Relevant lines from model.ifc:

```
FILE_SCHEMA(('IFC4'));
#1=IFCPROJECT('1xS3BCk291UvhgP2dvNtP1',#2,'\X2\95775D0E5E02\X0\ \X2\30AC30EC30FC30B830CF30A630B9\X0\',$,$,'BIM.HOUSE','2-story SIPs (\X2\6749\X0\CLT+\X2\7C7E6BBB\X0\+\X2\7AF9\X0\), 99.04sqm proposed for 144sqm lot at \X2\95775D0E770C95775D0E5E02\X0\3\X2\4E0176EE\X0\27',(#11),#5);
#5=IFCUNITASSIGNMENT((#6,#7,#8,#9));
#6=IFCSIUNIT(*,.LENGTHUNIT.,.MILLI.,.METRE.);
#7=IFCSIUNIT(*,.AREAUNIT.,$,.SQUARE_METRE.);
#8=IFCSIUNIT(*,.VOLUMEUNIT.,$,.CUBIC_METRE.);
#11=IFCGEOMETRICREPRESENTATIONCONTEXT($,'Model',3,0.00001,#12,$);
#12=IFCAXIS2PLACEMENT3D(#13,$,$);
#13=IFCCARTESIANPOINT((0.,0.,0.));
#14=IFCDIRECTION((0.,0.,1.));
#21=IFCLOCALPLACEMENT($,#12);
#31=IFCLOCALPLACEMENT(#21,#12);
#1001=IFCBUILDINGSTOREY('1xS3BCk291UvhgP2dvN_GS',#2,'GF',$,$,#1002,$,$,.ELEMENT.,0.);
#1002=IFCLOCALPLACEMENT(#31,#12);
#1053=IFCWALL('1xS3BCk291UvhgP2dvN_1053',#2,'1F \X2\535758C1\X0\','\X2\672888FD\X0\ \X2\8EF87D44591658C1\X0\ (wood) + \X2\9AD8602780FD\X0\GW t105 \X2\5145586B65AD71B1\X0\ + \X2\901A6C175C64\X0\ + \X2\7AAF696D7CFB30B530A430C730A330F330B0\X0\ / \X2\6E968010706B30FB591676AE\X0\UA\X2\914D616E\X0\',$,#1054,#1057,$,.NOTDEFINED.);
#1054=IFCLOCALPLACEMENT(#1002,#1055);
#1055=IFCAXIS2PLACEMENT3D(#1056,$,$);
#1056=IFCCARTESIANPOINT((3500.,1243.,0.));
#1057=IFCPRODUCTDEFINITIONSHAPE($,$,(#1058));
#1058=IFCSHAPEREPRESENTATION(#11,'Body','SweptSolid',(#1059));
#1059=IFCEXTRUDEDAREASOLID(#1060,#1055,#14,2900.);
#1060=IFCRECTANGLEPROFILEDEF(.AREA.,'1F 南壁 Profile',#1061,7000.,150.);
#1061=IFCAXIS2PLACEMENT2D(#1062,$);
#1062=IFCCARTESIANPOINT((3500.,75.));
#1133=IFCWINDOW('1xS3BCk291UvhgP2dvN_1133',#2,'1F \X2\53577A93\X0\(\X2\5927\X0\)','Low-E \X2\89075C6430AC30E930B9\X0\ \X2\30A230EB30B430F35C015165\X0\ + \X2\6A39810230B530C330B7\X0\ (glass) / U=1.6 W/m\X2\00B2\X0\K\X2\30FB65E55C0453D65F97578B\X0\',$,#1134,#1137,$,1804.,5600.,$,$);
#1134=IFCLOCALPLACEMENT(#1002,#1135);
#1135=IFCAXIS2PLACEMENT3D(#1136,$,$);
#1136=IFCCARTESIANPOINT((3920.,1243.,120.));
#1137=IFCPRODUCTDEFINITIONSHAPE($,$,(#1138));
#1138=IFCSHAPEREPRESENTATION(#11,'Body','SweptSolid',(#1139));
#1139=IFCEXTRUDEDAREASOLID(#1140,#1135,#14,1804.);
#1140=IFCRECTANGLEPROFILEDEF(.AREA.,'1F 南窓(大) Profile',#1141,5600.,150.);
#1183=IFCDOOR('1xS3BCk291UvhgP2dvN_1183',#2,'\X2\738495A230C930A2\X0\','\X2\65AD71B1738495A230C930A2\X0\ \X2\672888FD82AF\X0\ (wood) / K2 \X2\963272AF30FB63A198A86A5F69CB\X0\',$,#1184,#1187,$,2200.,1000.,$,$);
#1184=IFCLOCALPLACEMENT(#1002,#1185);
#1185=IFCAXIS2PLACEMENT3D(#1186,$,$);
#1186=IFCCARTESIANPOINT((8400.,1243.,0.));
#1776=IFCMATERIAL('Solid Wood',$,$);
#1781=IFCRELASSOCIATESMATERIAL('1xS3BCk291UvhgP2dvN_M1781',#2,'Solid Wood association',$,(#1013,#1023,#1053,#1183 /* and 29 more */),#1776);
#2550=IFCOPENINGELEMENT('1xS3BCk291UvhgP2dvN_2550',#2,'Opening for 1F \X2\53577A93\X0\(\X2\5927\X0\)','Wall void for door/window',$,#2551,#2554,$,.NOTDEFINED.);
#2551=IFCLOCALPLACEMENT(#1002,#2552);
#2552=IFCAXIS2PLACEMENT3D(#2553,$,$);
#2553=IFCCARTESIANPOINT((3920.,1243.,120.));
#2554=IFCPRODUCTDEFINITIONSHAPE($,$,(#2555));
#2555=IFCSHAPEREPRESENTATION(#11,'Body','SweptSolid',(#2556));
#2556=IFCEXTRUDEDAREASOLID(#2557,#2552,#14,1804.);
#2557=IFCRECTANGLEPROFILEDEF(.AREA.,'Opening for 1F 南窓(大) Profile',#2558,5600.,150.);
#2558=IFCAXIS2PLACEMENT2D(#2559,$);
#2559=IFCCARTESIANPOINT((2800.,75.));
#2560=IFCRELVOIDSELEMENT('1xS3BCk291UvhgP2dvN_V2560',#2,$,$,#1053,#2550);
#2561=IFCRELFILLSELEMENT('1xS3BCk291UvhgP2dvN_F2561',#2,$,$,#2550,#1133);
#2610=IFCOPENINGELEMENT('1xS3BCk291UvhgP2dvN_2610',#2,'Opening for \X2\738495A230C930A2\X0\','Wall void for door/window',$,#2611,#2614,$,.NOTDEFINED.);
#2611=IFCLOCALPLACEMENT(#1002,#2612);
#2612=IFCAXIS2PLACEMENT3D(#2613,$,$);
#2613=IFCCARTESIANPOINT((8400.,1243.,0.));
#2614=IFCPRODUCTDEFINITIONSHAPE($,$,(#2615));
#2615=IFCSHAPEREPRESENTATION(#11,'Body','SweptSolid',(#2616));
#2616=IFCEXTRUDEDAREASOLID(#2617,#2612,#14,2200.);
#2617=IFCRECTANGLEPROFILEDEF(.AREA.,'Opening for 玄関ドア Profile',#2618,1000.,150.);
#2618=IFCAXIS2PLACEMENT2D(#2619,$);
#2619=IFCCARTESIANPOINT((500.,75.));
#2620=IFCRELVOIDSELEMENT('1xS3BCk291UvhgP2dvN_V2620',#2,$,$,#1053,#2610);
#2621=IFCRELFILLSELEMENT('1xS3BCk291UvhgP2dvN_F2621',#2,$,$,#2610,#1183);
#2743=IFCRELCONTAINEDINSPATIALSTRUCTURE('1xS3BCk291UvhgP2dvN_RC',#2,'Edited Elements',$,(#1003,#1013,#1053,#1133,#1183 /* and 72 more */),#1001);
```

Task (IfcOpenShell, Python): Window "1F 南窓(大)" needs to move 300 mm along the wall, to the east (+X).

```python
import ifcopenshell
import ifcopenshell.api.geometry
import ifcopenshell.util.placement

model = ifcopenshell.open("model.ifc")

window = model.by_guid("1xS3BCk291UvhgP2dvN_1133")
opening = window.FillsVoids[0].RelatingOpeningElement
wall = opening.VoidsElements[0].RelatingBuildingElement

wall_matrix = ifcopenshell.util.placement.get_local_placement(wall.ObjectPlacement)
shift = wall_matrix[:3, 0] * 300.0
before = ifcopenshell.util.placement.get_local_placement(window.ObjectPlacement)[:3, 3].copy()

# The window is not placed relative to its opening, so move both.
for product in (opening, window):
    matrix = ifcopenshell.util.placement.get_local_placement(product.ObjectPlacement)
    matrix[:3, 3] += shift
    ifcopenshell.api.geometry.edit_object_placement(model, product=product, matrix=matrix, is_si=False)

after = ifcopenshell.util.placement.get_local_placement(window.ObjectPlacement)[:3, 3]
print("window moved by", (after - before).round(3) + 0.0)

model.write("model_updated.ifc")
```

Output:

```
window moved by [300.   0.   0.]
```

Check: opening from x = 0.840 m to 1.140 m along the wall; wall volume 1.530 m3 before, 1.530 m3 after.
